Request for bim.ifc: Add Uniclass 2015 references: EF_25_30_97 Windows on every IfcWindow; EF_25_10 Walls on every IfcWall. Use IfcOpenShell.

First a look at what the model holds.

```python
import ifcopenshell

model = ifcopenshell.open("bim.ifc")
print(model.schema)
print("classifications:", [c.Name for c in model.by_type("IfcClassification")])
for ifc_class in ("IfcDoor", "IfcRoof", "IfcStair", "IfcWall", "IfcWindow"):
    print(ifc_class, len(model.by_type(ifc_class)))
```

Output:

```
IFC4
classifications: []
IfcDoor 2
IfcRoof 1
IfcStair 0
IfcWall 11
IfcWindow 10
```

```python
import ifcopenshell
import ifcopenshell.api.classification

model = ifcopenshell.open("bim.ifc")

system = ifcopenshell.api.classification.add_classification(model, classification="Uniclass 2015")

codes = {
    "IfcWindow": ("EF_25_30_97", "Windows"),
    "IfcWall": ("EF_25_10", "Walls"),
}
for ifc_class, (code, name) in codes.items():
    products = model.by_type(ifc_class)
    ifcopenshell.api.classification.add_reference(
        model, products=products, classification=system, identification=code, name=name
    )
    print(code, len(products))

model.write("bim_rev.ifc")
```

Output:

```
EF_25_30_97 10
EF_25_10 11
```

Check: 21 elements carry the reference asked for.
